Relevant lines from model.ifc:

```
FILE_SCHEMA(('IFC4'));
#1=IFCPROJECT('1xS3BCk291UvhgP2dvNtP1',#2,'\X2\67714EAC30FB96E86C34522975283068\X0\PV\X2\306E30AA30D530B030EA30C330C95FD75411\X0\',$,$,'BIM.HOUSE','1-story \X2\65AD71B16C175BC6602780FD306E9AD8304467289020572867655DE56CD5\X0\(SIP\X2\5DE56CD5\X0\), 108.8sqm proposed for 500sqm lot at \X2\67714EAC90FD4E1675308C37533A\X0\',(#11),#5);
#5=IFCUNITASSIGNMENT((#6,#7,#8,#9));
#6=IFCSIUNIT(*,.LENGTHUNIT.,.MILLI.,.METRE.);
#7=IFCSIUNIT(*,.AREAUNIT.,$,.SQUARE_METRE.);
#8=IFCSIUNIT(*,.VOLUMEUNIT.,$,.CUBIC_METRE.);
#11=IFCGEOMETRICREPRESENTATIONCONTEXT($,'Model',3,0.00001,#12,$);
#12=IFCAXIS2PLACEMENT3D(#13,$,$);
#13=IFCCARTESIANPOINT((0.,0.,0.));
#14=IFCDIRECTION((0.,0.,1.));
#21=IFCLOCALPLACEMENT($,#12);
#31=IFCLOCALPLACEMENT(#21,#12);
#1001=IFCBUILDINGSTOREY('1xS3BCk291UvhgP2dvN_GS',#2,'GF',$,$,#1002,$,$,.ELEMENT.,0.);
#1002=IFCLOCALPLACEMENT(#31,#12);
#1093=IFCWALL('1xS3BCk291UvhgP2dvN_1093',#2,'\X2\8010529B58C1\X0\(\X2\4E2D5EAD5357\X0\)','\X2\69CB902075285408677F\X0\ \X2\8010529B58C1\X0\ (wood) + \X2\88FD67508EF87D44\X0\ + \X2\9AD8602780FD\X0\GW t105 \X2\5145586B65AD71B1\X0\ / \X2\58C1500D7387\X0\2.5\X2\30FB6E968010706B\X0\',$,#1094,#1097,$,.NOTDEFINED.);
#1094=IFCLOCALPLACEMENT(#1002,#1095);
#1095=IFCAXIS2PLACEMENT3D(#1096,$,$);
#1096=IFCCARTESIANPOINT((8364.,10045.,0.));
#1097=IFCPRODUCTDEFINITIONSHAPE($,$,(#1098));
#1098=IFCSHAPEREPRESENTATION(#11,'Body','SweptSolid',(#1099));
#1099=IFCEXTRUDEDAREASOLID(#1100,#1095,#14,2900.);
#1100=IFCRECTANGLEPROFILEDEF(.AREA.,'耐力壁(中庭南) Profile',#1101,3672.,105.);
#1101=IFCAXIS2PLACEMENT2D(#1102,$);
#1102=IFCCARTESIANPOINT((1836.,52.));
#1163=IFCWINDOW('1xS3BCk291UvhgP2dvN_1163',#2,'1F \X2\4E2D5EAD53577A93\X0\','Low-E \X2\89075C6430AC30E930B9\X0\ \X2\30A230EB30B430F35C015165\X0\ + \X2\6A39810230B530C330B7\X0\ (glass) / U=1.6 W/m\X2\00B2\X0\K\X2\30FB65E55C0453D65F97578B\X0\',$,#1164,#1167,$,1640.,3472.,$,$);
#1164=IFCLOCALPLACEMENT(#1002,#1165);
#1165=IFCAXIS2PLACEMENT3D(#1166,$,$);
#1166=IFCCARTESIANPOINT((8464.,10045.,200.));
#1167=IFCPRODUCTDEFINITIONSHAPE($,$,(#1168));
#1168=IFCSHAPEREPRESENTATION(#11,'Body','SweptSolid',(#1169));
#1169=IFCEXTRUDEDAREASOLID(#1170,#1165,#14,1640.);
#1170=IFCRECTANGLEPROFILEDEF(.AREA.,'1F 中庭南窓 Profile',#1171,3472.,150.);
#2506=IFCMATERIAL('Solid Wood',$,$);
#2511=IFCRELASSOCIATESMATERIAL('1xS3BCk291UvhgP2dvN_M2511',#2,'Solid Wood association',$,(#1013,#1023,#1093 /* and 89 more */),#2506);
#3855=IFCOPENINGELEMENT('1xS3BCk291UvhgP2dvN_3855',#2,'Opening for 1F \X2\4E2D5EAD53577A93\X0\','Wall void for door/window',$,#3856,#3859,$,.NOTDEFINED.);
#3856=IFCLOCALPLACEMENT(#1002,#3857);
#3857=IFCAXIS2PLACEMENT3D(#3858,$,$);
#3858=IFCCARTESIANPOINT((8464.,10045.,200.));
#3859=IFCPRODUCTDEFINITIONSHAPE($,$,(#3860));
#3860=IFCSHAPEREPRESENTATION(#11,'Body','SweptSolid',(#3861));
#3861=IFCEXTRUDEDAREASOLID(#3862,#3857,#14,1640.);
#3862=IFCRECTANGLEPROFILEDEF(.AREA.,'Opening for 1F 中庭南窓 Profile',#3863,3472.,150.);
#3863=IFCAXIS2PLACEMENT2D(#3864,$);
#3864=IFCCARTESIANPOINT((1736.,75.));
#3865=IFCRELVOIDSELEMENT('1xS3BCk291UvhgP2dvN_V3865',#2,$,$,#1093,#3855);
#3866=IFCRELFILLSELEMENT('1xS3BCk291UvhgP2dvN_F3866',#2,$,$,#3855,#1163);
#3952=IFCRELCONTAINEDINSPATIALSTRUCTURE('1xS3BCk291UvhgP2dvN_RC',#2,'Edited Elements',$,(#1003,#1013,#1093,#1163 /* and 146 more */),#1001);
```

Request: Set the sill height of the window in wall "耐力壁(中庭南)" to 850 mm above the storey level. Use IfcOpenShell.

```python
import numpy as np
import ifcopenshell
import ifcopenshell.api.geometry
import ifcopenshell.geom
import ifcopenshell.util.element
import ifcopenshell.util.placement
import ifcopenshell.util.shape
import ifcopenshell.util.unit

model = ifcopenshell.open("model.ifc")
unit_scale = ifcopenshell.util.unit.calculate_unit_scale(model)

window = model.by_guid("1xS3BCk291UvhgP2dvN_1163")
opening = window.FillsVoids[0].RelatingOpeningElement
storey = ifcopenshell.util.element.get_container(window, ifc_class="IfcBuildingStorey")
level = ifcopenshell.util.placement.get_local_placement(storey.ObjectPlacement)[2, 3]

# The opening's origin need not be at the sill, so measure its lowest point.
shape = ifcopenshell.geom.create_shape(ifcopenshell.geom.settings(), opening)
bottom = ifcopenshell.util.shape.get_shape_bottom_elevation(shape, shape.geometry) / unit_scale
dz = level + 0.85 / unit_scale - bottom

shift = np.array([0.0, 0.0, dz])
# The window is not placed relative to its opening, so move both.
for product in (opening, window):
    matrix = ifcopenshell.util.placement.get_local_placement(product.ObjectPlacement)
    matrix[:3, 3] += shift
    ifcopenshell.api.geometry.edit_object_placement(model, product=product, matrix=matrix, is_si=False)

print(f"moved by {dz * unit_scale:+.3f} m")

model.write("model_v2.ifc")
```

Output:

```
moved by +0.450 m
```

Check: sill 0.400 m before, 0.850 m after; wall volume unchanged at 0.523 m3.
